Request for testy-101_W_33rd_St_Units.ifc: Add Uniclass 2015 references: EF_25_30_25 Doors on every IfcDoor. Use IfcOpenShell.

First a look at what the model holds.

```python
import ifcopenshell

model = ifcopenshell.open("testy-101_W_33rd_St_Units.ifc")
print(model.schema)
print("classifications:", [c.Name for c in model.by_type("IfcClassification")])
for ifc_class in ("IfcDoor", "IfcRoof", "IfcStair", "IfcWall", "IfcWindow"):
    print(ifc_class, len(model.by_type(ifc_class)))
```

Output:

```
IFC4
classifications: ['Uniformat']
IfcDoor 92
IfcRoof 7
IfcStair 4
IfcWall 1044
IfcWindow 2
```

```python
import ifcopenshell
import ifcopenshell.api.classification

model = ifcopenshell.open("testy-101_W_33rd_St_Units.ifc")

system = ifcopenshell.api.classification.add_classification(model, classification="Uniclass 2015")

codes = {
    "IfcDoor": ("EF_25_30_25", "Doors"),
}
for ifc_class, (code, name) in codes.items():
    products = model.by_type(ifc_class)
    ifcopenshell.api.classification.add_reference(
        model, products=products, classification=system, identification=code, name=name
    )
    print(code, len(products))

model.write("testy-101_W_33rd_St_Units_rev.ifc")
```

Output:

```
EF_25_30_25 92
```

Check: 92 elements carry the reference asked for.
